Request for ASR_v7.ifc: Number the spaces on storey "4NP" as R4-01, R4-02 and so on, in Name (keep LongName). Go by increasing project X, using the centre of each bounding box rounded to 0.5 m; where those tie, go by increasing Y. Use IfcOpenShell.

First a look at what the model holds.

```python
import ifcopenshell
import ifcopenshell.util.element
import ifcopenshell.util.placement

model = ifcopenshell.open("ASR_v7.ifc")
print(model.schema)
storey = next(s for s in model.by_type("IfcBuildingStorey") if s.Name == "4NP")
spaces = [e for e in ifcopenshell.util.element.get_decomposition(storey) if e.is_a("IfcSpace")]
for e in sorted(spaces, key=lambda e: e.id()):
    origin = ifcopenshell.util.placement.get_local_placement(e.ObjectPlacement)[:3, 3]
    print(e.id(), e.Name, e.LongName, origin.round(2) + 0.0, sep=" | ")
```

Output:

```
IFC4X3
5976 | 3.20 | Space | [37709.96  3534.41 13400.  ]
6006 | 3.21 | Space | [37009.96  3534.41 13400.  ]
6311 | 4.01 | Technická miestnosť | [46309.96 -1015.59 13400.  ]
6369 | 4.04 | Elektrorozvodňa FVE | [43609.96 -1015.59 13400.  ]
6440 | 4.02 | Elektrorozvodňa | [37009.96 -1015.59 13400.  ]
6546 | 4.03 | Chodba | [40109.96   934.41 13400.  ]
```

```python
import ifcopenshell
import ifcopenshell.geom
import ifcopenshell.util.element
import ifcopenshell.util.shape

model = ifcopenshell.open("ASR_v7.ifc")
settings = ifcopenshell.geom.settings()
settings.set("use-world-coords", True)


def centre(element):
    shape = ifcopenshell.geom.create_shape(settings, element)
    return ifcopenshell.util.shape.get_bbox_centroid(shape.geometry)


storey = next(s for s in model.by_type("IfcBuildingStorey") if s.Name == "4NP")
spaces = [e for e in ifcopenshell.util.element.get_decomposition(storey) if e.is_a("IfcSpace")]

# Insertion points can sit at a corner or the storey origin, so sort by the geometry (in metres).
centres = {e: centre(e) for e in spaces}
spaces.sort(key=lambda e: (round(centres[e][0] / 0.5), centres[e][1]))

for i, e in enumerate(spaces, start=1):
    number = f"R4-{i:02d}"
    e.Name = number
    print(e.id(), number)

model.write("ASR_v7_rev.ifc")
```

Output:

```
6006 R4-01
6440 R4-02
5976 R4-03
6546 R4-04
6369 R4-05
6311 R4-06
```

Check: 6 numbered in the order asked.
